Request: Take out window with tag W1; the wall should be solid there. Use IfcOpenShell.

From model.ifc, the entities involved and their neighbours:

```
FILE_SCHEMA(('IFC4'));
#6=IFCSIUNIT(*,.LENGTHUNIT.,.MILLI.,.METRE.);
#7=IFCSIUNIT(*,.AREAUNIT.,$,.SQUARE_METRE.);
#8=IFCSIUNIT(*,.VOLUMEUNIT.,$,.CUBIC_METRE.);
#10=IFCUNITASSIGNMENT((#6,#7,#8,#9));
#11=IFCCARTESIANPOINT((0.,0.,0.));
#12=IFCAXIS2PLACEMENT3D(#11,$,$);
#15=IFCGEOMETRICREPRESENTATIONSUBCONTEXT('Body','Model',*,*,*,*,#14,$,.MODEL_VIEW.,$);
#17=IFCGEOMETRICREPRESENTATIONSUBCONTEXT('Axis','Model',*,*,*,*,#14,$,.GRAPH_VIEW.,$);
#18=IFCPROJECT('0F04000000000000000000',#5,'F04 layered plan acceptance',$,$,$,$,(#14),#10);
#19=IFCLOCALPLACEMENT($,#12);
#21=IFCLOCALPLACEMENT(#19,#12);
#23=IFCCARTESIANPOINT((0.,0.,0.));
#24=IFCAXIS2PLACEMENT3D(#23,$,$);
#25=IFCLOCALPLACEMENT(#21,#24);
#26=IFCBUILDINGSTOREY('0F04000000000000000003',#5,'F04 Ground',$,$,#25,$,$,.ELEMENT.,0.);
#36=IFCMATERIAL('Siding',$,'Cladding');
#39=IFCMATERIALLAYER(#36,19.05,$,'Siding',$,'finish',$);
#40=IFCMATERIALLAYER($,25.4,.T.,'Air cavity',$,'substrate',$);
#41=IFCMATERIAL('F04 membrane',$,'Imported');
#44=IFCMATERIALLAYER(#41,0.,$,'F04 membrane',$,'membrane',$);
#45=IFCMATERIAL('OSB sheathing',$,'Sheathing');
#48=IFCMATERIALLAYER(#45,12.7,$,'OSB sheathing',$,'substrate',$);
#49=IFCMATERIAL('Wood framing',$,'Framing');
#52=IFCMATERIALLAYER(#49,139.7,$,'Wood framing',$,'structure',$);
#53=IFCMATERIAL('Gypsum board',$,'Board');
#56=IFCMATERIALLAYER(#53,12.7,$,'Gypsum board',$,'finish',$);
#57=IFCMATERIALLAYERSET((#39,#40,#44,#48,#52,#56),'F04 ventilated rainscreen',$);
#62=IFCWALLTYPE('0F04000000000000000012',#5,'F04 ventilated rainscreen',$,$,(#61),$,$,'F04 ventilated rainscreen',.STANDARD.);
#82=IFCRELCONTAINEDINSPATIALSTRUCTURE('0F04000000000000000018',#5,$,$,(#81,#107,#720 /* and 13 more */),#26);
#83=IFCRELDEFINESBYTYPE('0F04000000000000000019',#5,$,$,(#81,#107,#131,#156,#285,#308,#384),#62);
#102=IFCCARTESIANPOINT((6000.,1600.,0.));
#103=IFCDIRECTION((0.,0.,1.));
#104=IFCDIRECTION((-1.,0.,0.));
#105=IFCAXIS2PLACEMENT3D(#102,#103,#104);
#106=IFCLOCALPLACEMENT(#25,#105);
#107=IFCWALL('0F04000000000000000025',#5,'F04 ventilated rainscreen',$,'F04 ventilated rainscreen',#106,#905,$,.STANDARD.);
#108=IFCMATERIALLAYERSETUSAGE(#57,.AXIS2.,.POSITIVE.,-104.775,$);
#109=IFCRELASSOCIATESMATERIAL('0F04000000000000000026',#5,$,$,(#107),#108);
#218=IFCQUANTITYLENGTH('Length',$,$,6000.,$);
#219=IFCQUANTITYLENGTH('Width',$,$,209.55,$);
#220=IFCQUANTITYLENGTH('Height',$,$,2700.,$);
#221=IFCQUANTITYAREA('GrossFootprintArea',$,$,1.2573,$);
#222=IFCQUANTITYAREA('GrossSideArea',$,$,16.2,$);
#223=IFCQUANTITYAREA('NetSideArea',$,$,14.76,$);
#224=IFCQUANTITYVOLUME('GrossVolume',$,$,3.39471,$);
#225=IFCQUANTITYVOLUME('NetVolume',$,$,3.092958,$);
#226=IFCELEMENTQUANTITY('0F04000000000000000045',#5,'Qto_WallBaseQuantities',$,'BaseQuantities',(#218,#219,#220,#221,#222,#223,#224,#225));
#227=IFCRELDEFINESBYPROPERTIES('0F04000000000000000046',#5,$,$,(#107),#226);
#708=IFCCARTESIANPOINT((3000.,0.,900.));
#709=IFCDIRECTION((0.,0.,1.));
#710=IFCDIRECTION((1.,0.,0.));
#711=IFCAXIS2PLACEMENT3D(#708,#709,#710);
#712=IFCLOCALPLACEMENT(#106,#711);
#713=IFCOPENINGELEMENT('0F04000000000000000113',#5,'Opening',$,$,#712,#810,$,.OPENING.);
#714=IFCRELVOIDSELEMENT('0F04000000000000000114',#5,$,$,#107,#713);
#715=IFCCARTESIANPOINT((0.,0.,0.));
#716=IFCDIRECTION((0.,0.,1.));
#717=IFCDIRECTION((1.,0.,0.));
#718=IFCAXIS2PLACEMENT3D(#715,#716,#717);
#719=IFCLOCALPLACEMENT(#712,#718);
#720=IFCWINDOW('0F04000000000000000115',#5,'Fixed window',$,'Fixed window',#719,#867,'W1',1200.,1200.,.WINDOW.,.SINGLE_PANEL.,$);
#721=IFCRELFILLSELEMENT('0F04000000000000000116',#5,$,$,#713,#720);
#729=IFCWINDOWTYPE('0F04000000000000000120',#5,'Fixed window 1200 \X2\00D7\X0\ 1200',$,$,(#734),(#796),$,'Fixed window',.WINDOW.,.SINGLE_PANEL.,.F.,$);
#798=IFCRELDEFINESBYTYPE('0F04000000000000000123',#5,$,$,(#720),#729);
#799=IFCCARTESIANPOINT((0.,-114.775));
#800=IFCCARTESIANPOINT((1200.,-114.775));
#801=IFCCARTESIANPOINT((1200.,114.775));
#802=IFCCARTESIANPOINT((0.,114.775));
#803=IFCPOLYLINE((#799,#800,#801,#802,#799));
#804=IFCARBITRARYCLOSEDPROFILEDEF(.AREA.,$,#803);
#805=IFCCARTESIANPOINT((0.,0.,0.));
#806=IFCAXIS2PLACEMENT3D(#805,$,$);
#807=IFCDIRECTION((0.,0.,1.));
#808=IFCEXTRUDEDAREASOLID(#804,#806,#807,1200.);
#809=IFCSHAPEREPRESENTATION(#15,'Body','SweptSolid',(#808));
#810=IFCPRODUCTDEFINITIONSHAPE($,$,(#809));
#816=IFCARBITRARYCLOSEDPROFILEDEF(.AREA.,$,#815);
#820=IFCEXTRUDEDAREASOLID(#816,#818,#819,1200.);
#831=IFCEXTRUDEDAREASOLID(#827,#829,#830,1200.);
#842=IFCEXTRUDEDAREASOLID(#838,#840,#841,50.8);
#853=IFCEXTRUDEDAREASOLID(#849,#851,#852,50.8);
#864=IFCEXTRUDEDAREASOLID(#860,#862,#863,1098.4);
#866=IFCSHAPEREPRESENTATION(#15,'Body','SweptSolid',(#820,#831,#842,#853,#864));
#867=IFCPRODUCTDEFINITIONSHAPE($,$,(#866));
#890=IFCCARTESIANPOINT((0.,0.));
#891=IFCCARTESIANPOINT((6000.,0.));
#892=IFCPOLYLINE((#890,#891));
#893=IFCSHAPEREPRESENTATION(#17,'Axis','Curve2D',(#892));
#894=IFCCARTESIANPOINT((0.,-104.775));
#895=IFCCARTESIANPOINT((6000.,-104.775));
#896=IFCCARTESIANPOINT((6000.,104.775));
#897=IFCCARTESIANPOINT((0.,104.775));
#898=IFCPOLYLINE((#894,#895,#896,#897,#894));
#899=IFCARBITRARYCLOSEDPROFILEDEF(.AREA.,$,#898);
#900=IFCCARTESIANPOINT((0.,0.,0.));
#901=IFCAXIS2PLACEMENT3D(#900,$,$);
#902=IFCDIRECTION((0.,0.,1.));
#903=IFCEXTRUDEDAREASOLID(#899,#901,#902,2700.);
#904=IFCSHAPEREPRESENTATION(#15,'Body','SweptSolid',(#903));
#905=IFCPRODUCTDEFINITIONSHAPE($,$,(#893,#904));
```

```python
import ifcopenshell
import ifcopenshell.api.feature
import ifcopenshell.api.pset
import ifcopenshell.api.root
import ifcopenshell.geom
import ifcopenshell.util.element
import ifcopenshell.util.shape
import ifcopenshell.util.unit

model = ifcopenshell.open("model.ifc")
area_scale = ifcopenshell.util.unit.calculate_unit_scale(model, "AREAUNIT")
volume_scale = ifcopenshell.util.unit.calculate_unit_scale(model, "VOLUMEUNIT")
settings = ifcopenshell.geom.settings()


def volume(element):
    """Net volume in cubic metres, openings subtracted."""
    shape = ifcopenshell.geom.create_shape(settings, element)
    return ifcopenshell.util.shape.get_volume(shape.geometry)


window = model.by_guid("0F04000000000000000115")
opening = window.FillsVoids[0].RelatingOpeningElement
wall = opening.VoidsElements[0].RelatingBuildingElement
before = volume(wall)

ifcopenshell.api.root.remove_product(model, product=window)
ifcopenshell.api.feature.remove_feature(model, feature=opening)

after = volume(wall)
thickness = 0.2096  # wall thickness in metres

# Update the wall's stored quantities.
qto = model.by_id(ifcopenshell.util.element.get_pset(wall, "Qto_WallBaseQuantities", should_inherit=False)["id"])
ifcopenshell.api.pset.edit_qto(model, qto=qto, properties={
    "NetSideArea": after / thickness / area_scale,
    "NetVolume": after / volume_scale,
})

print(f"wall volume {before:.3f} -> {after:.3f} m3")

model.write("model_edited.ifc")
```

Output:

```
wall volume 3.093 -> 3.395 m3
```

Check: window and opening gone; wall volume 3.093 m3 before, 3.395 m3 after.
